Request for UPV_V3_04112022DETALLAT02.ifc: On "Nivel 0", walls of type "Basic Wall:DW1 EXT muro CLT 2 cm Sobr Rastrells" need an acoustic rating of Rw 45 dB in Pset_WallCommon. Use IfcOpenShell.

First a look at what the model holds.

```python
import ifcopenshell
import ifcopenshell.util.element

model = ifcopenshell.open("UPV_V3_04112022DETALLAT02.ifc")
print(model.schema)
storey = next(s for s in model.by_type("IfcBuildingStorey") if s.Name == "Nivel 0")
walls = [e for e in ifcopenshell.util.element.get_decomposition(storey) if e.is_a("IfcWall")]
seen = {}
for e in walls:
    element_type = ifcopenshell.util.element.get_type(e)
    key = (element_type.Name if element_type != e and element_type else None, ifcopenshell.util.element.get_pset(e, "Pset_WallCommon", "AcousticRating"))
    seen[key] = seen.get(key, 0) + 1
for (name, value), count in sorted(seen.items(), key=str):
    print(count, "x", name, "|", value)
```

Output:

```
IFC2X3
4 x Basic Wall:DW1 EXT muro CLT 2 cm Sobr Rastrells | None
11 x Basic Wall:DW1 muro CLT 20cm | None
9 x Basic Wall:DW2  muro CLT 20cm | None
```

```python
import ifcopenshell
import ifcopenshell.api.pset
import ifcopenshell.util.element

model = ifcopenshell.open("UPV_V3_04112022DETALLAT02.ifc")

storey = next(s for s in model.by_type("IfcBuildingStorey") if s.Name == "Nivel 0")
walls = [e for e in ifcopenshell.util.element.get_decomposition(storey) if e.is_a("IfcWall")]

count = 0
for e in walls:
    element_type = ifcopenshell.util.element.get_type(e)
    if element_type in (None, e) or element_type.Name != "Basic Wall:DW1 EXT muro CLT 2 cm Sobr Rastrells":
        continue
    # add_pset returns the element's existing set when there is one.
    pset = ifcopenshell.api.pset.add_pset(model, product=e, name="Pset_WallCommon")
    ifcopenshell.api.pset.edit_pset(model, pset=pset, properties={"AcousticRating": "Rw 45 dB"})
    count += 1

print(count, "walls updated")

model.write("UPV_V3_04112022DETALLAT02-out.ifc")
```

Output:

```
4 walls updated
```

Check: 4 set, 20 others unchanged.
